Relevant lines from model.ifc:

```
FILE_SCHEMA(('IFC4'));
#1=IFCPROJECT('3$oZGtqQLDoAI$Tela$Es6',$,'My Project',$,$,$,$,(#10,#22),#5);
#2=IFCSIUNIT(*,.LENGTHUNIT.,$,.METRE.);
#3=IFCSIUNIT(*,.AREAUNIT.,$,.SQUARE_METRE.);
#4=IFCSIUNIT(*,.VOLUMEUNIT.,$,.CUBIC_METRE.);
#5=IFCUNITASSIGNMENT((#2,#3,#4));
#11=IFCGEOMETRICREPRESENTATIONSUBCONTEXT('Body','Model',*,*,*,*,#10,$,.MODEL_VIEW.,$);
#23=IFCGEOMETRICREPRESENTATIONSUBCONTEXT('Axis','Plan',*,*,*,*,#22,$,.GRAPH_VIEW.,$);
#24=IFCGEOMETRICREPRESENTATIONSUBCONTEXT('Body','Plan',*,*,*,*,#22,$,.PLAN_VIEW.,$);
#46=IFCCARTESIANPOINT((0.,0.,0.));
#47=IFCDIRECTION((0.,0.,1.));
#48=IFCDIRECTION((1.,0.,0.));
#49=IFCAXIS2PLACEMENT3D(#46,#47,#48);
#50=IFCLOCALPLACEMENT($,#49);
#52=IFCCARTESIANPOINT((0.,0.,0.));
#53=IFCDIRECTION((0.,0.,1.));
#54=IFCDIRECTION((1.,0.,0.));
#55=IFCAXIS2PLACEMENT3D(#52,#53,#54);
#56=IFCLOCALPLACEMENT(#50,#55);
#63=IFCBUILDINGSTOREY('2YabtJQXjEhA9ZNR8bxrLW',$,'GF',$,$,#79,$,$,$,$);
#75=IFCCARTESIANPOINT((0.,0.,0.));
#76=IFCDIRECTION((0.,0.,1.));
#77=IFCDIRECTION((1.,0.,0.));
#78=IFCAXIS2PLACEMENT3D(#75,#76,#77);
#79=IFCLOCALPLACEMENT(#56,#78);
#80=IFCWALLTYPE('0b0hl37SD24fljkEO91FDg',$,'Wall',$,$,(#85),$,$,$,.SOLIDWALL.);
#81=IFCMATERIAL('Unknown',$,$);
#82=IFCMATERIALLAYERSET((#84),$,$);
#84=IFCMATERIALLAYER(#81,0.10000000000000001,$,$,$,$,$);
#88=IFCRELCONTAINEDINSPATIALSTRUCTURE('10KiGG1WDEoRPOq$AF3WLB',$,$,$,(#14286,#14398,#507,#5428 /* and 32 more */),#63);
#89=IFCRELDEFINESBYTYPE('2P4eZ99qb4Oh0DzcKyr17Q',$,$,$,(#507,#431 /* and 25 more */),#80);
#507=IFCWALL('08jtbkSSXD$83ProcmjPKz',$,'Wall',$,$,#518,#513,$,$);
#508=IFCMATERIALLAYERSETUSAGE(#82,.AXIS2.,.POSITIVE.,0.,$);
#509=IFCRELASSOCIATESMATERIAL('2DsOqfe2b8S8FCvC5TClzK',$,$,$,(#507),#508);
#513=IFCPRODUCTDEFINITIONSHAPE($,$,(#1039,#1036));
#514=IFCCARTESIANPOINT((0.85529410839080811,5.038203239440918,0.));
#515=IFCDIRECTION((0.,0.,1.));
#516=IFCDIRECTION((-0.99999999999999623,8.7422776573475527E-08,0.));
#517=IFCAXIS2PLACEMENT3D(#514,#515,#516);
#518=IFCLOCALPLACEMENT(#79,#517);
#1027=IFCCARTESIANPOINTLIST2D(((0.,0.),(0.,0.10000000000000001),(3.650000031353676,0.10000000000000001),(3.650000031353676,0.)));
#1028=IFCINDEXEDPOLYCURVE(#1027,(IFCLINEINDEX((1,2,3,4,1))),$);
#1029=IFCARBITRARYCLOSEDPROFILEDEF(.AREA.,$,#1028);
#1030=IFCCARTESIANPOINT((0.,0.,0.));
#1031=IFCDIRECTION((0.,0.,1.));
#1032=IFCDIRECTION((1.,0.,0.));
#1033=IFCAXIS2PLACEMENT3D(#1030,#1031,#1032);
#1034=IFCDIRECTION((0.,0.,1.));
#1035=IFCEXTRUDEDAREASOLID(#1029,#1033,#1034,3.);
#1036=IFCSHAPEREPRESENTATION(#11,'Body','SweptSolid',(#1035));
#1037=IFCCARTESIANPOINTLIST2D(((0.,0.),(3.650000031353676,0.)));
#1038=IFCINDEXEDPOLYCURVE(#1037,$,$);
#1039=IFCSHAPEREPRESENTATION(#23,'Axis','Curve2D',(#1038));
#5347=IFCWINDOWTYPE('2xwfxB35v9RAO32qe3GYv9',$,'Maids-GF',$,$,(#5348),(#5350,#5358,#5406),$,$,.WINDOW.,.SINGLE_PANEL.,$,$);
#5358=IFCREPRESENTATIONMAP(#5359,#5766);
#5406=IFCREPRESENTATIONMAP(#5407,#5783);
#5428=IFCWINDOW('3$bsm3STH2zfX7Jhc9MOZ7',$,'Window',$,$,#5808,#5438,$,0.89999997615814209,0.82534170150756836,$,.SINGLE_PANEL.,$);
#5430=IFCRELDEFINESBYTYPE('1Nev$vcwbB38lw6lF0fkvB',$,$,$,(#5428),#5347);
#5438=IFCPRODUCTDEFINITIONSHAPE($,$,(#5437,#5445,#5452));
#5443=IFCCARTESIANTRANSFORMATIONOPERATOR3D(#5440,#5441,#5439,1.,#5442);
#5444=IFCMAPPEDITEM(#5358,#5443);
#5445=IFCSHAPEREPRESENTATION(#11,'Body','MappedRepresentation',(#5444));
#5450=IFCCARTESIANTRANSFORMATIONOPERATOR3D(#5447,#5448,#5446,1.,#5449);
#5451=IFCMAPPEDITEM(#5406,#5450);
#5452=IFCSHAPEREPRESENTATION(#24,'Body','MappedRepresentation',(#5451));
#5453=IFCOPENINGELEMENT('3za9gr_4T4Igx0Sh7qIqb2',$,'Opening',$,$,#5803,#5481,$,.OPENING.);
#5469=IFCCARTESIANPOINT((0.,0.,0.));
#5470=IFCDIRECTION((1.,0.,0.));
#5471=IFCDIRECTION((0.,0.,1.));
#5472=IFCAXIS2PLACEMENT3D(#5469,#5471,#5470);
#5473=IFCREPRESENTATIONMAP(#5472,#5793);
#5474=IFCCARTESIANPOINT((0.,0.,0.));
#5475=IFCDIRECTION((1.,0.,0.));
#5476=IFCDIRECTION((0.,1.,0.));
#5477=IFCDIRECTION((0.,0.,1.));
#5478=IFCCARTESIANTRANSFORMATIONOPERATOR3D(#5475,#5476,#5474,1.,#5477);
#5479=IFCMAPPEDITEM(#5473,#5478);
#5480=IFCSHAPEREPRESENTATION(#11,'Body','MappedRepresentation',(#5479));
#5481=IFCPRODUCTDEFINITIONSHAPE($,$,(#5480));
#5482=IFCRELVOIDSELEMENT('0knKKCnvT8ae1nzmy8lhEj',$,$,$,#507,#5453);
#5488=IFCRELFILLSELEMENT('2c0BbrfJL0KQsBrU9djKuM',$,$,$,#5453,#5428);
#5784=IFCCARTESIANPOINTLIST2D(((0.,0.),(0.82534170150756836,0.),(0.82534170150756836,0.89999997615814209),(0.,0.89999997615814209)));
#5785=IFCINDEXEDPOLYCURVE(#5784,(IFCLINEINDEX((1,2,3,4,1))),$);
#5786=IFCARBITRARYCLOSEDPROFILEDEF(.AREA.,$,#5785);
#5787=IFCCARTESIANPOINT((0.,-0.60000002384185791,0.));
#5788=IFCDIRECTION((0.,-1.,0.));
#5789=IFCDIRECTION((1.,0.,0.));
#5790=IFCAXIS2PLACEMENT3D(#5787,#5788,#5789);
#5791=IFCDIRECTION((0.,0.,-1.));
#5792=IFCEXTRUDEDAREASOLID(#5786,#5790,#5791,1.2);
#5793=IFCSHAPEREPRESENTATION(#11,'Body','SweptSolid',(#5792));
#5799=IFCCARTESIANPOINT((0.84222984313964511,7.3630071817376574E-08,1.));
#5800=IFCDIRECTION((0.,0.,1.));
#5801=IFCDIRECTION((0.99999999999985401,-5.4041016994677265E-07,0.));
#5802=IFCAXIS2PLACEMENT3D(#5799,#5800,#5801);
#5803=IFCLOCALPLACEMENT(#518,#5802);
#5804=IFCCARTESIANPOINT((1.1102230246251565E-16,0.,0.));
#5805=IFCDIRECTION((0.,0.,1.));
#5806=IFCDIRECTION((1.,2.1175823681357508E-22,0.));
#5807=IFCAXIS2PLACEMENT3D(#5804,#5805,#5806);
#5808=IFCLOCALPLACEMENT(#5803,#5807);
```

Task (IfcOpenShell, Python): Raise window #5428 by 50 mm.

```python
import numpy as np
import ifcopenshell
import ifcopenshell.api.geometry
import ifcopenshell.util.placement
import ifcopenshell.util.unit

model = ifcopenshell.open("model.ifc")
unit_scale = ifcopenshell.util.unit.calculate_unit_scale(model)

window = model.by_id(5428)
opening = window.FillsVoids[0].RelatingOpeningElement
dz = 0.05

shift = np.array([0.0, 0.0, dz])
# The window is placed relative to its opening, so it follows when the opening moves.
matrix = ifcopenshell.util.placement.get_local_placement(opening.ObjectPlacement)
matrix[:3, 3] += shift
ifcopenshell.api.geometry.edit_object_placement(
    model, product=opening, matrix=matrix, is_si=False, should_transform_children=True
)

print(f"moved by {dz * unit_scale:+.3f} m")

model.write("model_rev.ifc")
```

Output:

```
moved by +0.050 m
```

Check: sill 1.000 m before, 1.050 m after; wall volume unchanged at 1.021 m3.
